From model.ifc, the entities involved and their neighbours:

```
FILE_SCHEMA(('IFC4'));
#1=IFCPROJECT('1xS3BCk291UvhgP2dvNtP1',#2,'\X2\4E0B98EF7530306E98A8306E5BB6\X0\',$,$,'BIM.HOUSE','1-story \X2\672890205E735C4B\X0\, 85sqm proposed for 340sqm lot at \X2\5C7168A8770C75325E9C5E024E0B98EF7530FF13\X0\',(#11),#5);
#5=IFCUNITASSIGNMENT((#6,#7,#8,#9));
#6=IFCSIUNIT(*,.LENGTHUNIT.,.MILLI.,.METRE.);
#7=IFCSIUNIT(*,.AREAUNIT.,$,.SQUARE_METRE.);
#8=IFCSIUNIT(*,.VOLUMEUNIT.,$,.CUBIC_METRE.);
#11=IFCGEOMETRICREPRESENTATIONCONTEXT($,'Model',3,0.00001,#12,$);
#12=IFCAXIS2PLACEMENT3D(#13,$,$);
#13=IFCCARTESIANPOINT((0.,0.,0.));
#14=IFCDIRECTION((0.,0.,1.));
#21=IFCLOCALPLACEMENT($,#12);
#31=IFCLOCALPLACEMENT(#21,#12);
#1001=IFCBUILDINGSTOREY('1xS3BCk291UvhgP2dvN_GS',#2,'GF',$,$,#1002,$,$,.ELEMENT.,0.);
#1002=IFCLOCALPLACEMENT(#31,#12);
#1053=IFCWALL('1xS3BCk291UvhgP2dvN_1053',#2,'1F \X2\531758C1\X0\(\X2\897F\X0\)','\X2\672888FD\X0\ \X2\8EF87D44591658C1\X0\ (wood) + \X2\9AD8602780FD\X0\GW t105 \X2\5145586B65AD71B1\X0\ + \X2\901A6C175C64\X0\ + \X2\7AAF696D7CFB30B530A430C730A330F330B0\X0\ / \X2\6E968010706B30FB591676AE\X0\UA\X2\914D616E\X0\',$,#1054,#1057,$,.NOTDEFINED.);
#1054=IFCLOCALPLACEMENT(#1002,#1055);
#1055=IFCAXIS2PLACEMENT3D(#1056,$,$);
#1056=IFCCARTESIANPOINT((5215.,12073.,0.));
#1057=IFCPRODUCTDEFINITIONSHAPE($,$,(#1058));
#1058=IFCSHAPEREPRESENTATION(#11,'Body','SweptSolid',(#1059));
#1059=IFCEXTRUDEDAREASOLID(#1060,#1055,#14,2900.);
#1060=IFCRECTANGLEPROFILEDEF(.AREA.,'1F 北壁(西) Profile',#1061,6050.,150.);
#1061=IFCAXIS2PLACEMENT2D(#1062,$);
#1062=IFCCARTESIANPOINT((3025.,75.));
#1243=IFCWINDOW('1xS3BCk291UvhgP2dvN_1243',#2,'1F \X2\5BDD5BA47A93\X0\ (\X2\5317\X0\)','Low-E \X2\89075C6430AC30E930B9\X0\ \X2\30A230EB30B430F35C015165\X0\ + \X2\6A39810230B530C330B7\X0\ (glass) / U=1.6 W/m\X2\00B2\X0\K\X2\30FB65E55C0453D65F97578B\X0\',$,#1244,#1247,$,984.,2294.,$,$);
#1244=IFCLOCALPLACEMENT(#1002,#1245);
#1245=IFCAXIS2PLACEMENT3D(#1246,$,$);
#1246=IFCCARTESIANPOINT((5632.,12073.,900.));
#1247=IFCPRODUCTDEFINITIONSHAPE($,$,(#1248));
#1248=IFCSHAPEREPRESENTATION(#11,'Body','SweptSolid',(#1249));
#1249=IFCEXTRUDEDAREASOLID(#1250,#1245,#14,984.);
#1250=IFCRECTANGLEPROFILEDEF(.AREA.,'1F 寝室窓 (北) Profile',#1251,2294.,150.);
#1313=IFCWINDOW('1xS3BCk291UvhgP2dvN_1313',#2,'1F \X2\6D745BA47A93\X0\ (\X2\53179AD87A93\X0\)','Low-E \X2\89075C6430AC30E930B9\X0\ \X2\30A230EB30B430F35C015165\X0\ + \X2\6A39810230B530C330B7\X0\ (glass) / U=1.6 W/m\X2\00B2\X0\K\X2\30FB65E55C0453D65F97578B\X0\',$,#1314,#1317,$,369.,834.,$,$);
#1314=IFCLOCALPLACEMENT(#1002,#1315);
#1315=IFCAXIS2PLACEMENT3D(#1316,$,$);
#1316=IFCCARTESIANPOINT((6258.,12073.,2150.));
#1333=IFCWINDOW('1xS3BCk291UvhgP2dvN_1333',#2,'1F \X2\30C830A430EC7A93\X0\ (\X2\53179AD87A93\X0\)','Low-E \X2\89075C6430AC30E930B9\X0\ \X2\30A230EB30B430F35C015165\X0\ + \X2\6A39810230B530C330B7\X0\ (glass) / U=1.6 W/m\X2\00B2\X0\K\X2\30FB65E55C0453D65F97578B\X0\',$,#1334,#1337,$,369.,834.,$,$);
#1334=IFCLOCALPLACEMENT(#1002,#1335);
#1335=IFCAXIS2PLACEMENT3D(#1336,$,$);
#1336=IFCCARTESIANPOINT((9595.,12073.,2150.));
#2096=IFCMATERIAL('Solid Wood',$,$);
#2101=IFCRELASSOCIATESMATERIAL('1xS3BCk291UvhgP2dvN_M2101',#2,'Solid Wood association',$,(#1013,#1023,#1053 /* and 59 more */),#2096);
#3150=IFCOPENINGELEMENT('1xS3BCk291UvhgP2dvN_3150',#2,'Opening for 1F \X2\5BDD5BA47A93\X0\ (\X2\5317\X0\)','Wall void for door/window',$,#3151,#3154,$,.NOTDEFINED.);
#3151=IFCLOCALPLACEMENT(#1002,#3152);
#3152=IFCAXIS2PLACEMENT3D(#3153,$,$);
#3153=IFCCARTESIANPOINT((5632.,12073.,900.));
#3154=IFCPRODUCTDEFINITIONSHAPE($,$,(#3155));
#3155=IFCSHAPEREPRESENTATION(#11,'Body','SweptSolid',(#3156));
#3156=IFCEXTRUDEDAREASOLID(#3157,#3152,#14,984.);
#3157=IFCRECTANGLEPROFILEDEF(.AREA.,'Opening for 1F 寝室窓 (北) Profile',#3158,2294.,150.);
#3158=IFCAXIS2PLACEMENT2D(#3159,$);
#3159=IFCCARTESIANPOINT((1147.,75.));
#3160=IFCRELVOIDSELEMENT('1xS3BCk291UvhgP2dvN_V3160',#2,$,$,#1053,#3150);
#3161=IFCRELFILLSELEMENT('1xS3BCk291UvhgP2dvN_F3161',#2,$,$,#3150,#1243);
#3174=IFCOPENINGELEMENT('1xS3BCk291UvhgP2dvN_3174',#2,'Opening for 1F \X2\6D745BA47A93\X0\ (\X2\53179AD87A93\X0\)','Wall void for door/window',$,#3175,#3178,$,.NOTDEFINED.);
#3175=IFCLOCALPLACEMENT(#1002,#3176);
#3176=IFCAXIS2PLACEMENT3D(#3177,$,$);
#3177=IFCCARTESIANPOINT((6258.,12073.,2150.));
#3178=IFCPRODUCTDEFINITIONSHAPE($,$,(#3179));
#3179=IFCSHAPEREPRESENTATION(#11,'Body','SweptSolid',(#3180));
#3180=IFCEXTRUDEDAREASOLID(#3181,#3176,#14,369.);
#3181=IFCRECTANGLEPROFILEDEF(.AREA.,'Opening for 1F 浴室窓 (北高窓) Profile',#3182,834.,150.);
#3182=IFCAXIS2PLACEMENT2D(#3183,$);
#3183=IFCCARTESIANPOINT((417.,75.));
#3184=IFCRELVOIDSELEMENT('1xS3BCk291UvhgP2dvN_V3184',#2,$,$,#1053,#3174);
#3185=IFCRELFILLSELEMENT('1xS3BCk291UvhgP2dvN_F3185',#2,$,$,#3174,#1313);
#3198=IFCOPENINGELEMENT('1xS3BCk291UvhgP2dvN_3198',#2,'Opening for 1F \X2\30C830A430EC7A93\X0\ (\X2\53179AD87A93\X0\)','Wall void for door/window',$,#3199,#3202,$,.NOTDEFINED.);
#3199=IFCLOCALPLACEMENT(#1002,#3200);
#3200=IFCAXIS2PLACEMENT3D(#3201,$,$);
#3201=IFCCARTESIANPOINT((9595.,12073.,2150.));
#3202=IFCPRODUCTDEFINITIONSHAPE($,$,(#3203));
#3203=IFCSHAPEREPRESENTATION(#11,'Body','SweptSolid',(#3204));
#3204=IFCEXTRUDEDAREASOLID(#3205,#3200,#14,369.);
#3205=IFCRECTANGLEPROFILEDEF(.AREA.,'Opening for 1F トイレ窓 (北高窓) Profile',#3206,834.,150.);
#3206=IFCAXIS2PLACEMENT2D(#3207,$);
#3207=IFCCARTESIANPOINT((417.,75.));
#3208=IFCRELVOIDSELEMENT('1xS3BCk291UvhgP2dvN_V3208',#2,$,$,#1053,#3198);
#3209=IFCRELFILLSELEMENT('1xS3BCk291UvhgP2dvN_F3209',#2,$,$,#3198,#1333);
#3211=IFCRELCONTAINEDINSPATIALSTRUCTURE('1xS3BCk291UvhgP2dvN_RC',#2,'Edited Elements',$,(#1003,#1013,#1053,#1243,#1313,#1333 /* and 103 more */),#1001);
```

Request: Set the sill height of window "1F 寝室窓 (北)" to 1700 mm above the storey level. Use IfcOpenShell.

```python
import numpy as np
import ifcopenshell
import ifcopenshell.api.geometry
import ifcopenshell.geom
import ifcopenshell.util.element
import ifcopenshell.util.placement
import ifcopenshell.util.shape
import ifcopenshell.util.unit

model = ifcopenshell.open("model.ifc")
unit_scale = ifcopenshell.util.unit.calculate_unit_scale(model)

window = model.by_guid("1xS3BCk291UvhgP2dvN_1243")
opening = window.FillsVoids[0].RelatingOpeningElement
storey = ifcopenshell.util.element.get_container(window, ifc_class="IfcBuildingStorey")
level = ifcopenshell.util.placement.get_local_placement(storey.ObjectPlacement)[2, 3]

# The opening's origin need not be at the sill, so measure its lowest point.
shape = ifcopenshell.geom.create_shape(ifcopenshell.geom.settings(), opening)
bottom = ifcopenshell.util.shape.get_shape_bottom_elevation(shape, shape.geometry) / unit_scale
dz = level + 1700.0 - bottom

shift = np.array([0.0, 0.0, dz])
# The window is not placed relative to its opening, so move both.
for product in (opening, window):
    matrix = ifcopenshell.util.placement.get_local_placement(product.ObjectPlacement)
    matrix[:3, 3] += shift
    ifcopenshell.api.geometry.edit_object_placement(model, product=product, matrix=matrix, is_si=False)

print(f"moved by {dz * unit_scale:+.3f} m")

model.write("model-out.ifc")
```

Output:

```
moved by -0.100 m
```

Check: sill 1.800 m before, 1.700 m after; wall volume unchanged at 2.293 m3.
